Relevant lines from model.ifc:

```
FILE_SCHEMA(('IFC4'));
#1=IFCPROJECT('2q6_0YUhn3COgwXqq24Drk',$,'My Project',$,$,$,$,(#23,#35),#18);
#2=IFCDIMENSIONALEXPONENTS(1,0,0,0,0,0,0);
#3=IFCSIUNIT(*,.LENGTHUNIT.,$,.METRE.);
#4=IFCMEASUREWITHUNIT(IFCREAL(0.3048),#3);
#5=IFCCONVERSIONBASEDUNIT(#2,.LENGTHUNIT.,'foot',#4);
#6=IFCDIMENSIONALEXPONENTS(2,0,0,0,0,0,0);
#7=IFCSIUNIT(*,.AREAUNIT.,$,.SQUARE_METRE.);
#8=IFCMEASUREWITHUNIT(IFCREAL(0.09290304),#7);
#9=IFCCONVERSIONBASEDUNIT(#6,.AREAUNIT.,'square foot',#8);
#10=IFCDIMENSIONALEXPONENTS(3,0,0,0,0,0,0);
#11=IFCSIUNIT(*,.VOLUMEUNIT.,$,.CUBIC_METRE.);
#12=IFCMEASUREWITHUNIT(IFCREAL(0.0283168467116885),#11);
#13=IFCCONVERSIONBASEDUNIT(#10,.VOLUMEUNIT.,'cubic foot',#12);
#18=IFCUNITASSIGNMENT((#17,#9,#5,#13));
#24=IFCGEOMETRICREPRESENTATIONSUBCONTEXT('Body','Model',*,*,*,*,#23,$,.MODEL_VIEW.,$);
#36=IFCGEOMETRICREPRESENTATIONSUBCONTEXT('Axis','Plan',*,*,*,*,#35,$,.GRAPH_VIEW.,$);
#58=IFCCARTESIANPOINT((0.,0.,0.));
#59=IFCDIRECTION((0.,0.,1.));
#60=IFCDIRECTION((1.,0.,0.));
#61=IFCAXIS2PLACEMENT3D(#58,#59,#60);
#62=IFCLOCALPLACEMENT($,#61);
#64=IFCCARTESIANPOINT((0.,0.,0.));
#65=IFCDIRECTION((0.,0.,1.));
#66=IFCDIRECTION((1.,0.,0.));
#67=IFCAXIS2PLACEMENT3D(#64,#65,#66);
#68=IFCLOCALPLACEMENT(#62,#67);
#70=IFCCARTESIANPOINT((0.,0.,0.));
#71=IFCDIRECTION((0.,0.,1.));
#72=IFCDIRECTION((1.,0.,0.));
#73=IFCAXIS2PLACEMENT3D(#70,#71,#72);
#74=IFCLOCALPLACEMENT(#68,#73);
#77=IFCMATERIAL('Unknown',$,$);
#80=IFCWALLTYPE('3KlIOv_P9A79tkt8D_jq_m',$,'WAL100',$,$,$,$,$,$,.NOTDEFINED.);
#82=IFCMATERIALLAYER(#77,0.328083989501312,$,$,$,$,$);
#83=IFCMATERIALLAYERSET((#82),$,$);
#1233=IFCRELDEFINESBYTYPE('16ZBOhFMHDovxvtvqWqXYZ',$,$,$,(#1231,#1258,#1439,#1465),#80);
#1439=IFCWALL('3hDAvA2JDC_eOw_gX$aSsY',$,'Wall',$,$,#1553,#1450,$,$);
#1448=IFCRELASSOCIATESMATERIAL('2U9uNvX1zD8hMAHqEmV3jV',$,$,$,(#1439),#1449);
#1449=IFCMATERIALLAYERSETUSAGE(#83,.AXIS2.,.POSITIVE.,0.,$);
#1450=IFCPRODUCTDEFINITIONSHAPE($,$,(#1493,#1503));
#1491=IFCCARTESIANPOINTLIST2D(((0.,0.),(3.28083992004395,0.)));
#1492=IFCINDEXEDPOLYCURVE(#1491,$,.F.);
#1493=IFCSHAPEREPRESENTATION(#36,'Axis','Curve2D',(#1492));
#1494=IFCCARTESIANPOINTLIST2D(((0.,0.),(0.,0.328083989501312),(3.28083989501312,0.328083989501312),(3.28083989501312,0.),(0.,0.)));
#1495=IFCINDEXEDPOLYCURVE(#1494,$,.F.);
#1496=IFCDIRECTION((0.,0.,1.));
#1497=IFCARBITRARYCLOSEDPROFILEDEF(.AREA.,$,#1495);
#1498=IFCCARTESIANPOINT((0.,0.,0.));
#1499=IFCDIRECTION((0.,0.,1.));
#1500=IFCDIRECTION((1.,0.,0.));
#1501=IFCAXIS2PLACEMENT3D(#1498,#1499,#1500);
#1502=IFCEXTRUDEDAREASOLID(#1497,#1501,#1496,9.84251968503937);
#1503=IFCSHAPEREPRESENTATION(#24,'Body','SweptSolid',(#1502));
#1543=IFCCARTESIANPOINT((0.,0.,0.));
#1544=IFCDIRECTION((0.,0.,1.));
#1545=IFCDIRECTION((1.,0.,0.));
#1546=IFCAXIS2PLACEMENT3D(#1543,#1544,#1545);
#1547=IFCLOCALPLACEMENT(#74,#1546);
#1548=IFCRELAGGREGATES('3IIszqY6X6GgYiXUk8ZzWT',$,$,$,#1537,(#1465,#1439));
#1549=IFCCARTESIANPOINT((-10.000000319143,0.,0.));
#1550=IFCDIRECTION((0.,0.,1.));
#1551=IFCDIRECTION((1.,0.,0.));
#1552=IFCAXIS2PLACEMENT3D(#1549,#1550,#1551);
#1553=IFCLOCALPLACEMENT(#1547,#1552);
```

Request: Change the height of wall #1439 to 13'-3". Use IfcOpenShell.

```python
import ifcopenshell
import ifcopenshell.geom
import ifcopenshell.util.representation
import ifcopenshell.util.shape
import ifcopenshell.util.unit

model = ifcopenshell.open("model.ifc")
unit_scale = ifcopenshell.util.unit.calculate_unit_scale(model)
settings = ifcopenshell.geom.settings()


def volume(element):
    """Net volume in cubic metres, openings subtracted."""
    shape = ifcopenshell.geom.create_shape(settings, element)
    return ifcopenshell.util.shape.get_volume(shape.geometry)


wall = model.by_id(1439)
before = volume(wall)

body = ifcopenshell.util.representation.get_representation(wall, "Model", "Body")
solid = body.Items[0]
old_height = solid.Depth
solid.Depth = 159 * 0.0254 / unit_scale
after = volume(wall)

print(f"height {old_height:g} -> {solid.Depth:g}, volume {before:.3f} -> {after:.3f} m3")

model.write("model_edited.ifc")
```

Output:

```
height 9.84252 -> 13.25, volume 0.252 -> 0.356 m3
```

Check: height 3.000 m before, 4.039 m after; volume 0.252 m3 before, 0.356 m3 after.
